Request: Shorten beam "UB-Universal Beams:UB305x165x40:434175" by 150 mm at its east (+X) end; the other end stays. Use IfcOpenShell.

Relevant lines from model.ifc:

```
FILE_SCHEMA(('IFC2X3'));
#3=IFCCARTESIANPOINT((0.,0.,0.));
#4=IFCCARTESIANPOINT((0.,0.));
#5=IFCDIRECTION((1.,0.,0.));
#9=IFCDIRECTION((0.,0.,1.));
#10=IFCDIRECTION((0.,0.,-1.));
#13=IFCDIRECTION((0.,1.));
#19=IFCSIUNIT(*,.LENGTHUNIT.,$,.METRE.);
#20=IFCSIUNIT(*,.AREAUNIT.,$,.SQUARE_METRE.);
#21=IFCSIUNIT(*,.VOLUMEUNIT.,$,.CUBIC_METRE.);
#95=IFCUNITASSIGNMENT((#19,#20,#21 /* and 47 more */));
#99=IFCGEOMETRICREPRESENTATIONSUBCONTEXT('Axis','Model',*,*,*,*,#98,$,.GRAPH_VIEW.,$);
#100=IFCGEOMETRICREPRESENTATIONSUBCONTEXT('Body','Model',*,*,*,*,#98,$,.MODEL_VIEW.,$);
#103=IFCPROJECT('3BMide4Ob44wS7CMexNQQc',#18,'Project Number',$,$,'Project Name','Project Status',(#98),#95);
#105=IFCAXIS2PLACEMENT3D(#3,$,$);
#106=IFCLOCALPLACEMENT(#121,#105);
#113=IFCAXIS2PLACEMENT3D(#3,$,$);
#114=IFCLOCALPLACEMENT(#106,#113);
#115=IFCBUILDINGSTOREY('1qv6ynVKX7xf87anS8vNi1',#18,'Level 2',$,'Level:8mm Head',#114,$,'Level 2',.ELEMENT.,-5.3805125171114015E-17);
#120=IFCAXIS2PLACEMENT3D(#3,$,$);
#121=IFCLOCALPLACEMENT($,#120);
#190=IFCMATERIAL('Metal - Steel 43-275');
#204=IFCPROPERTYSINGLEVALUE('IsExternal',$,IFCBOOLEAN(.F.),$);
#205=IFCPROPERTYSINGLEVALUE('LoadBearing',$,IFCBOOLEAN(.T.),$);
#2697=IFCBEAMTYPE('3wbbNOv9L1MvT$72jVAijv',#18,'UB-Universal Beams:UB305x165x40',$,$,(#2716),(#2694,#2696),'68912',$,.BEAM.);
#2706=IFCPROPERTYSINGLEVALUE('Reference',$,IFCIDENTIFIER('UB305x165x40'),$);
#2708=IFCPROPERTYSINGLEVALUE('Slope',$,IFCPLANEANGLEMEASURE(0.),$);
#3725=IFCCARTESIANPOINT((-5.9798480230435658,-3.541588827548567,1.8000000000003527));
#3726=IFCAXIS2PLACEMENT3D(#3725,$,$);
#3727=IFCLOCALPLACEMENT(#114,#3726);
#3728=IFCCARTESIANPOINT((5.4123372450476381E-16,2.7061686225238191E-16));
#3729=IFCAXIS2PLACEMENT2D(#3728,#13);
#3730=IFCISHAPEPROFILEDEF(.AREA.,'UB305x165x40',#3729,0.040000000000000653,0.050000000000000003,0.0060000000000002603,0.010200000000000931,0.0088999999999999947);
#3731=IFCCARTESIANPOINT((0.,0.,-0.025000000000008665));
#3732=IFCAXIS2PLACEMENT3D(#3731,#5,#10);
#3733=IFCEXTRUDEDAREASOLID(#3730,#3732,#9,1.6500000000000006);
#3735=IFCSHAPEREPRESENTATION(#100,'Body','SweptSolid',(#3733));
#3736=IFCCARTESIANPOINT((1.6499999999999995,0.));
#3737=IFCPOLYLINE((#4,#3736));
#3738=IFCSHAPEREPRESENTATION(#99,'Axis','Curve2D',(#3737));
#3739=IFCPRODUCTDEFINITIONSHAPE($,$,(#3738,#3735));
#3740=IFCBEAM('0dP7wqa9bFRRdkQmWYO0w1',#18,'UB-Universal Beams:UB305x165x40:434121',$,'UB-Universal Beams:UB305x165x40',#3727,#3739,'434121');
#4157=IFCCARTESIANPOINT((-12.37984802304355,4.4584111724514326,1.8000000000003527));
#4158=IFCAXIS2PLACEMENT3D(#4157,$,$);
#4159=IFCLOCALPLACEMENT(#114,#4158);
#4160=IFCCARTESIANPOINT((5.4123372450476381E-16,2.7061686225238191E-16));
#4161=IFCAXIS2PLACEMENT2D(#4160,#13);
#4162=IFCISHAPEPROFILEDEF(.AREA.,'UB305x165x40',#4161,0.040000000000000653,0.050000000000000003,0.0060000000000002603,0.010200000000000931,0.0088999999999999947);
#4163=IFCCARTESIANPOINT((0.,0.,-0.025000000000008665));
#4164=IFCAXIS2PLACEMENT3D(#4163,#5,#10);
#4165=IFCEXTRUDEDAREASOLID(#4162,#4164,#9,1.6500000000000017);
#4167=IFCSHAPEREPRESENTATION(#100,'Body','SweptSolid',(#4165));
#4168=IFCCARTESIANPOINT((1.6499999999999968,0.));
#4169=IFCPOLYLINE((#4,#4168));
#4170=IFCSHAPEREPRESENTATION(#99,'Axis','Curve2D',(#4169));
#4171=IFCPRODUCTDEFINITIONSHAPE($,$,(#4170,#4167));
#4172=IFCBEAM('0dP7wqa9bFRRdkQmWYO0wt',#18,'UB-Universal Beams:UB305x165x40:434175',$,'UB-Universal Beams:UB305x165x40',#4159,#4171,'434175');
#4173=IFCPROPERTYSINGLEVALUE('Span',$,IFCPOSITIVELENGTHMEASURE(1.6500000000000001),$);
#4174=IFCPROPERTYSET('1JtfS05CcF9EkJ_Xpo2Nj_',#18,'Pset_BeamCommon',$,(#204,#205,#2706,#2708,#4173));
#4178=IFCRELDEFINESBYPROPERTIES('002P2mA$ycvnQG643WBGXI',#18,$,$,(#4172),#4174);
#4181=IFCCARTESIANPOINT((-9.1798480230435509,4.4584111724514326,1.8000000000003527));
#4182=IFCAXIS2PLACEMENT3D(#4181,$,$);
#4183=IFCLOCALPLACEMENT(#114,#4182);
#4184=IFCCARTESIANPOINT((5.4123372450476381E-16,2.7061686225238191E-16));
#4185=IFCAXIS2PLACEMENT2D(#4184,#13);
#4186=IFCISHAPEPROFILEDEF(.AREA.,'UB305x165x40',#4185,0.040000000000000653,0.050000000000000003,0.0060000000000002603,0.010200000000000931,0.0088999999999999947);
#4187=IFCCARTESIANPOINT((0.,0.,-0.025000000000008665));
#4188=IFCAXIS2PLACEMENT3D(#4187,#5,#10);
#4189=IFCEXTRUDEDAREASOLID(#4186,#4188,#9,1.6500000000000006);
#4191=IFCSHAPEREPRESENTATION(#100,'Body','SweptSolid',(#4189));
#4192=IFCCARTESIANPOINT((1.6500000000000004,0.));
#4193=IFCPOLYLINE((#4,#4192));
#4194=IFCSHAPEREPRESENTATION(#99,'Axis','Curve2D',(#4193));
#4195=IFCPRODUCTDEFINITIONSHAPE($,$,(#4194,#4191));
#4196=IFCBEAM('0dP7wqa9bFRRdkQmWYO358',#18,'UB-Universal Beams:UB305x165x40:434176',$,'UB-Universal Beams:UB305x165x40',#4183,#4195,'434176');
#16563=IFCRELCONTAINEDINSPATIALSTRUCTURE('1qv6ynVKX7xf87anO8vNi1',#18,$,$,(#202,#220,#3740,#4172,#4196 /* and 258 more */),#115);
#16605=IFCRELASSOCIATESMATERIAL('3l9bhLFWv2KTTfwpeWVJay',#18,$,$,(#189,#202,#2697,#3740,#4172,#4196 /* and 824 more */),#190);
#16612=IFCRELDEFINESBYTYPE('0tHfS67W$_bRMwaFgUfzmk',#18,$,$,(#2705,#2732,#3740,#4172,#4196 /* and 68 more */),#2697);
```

```python
import numpy as np
import ifcopenshell
import ifcopenshell.api.pset
import ifcopenshell.util.element
import ifcopenshell.util.representation
import ifcopenshell.util.unit

model = ifcopenshell.open("model.ifc")
unit_scale = ifcopenshell.util.unit.calculate_unit_scale(model)

member = model.by_id(4172)
change = -0.15 / unit_scale

# The extrusion runs towards the end named, so only its depth changes.
body = ifcopenshell.util.representation.get_representation(member, "Model", "Body")
solid = body.Items[0]
old_length = solid.Depth
solid.Depth += change

# Move the axis end point with it.
axis = next(r for r in member.Representation.Representations if r.RepresentationIdentifier == "Axis").Items[0]
start, end = (np.array(p.Coordinates) for p in axis.Points)
end = end + (end - start) / np.linalg.norm(end - start) * change
point = model.createIfcCartesianPoint(end.tolist())
axis.Points = [axis.Points[0], point]

# Update the stored length and volume.
pset = model.by_id(ifcopenshell.util.element.get_pset(member, "Pset_BeamCommon", should_inherit=False)["id"])
ifcopenshell.api.pset.edit_pset(model, pset=pset, properties={
    "Span": model.create_entity("IfcPositiveLengthMeasure", solid.Depth),
})

print(f"length {old_length:g} -> {solid.Depth:g}")

model.write("model_edited.ifc")
```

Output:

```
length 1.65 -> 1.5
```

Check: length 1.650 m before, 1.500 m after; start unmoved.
